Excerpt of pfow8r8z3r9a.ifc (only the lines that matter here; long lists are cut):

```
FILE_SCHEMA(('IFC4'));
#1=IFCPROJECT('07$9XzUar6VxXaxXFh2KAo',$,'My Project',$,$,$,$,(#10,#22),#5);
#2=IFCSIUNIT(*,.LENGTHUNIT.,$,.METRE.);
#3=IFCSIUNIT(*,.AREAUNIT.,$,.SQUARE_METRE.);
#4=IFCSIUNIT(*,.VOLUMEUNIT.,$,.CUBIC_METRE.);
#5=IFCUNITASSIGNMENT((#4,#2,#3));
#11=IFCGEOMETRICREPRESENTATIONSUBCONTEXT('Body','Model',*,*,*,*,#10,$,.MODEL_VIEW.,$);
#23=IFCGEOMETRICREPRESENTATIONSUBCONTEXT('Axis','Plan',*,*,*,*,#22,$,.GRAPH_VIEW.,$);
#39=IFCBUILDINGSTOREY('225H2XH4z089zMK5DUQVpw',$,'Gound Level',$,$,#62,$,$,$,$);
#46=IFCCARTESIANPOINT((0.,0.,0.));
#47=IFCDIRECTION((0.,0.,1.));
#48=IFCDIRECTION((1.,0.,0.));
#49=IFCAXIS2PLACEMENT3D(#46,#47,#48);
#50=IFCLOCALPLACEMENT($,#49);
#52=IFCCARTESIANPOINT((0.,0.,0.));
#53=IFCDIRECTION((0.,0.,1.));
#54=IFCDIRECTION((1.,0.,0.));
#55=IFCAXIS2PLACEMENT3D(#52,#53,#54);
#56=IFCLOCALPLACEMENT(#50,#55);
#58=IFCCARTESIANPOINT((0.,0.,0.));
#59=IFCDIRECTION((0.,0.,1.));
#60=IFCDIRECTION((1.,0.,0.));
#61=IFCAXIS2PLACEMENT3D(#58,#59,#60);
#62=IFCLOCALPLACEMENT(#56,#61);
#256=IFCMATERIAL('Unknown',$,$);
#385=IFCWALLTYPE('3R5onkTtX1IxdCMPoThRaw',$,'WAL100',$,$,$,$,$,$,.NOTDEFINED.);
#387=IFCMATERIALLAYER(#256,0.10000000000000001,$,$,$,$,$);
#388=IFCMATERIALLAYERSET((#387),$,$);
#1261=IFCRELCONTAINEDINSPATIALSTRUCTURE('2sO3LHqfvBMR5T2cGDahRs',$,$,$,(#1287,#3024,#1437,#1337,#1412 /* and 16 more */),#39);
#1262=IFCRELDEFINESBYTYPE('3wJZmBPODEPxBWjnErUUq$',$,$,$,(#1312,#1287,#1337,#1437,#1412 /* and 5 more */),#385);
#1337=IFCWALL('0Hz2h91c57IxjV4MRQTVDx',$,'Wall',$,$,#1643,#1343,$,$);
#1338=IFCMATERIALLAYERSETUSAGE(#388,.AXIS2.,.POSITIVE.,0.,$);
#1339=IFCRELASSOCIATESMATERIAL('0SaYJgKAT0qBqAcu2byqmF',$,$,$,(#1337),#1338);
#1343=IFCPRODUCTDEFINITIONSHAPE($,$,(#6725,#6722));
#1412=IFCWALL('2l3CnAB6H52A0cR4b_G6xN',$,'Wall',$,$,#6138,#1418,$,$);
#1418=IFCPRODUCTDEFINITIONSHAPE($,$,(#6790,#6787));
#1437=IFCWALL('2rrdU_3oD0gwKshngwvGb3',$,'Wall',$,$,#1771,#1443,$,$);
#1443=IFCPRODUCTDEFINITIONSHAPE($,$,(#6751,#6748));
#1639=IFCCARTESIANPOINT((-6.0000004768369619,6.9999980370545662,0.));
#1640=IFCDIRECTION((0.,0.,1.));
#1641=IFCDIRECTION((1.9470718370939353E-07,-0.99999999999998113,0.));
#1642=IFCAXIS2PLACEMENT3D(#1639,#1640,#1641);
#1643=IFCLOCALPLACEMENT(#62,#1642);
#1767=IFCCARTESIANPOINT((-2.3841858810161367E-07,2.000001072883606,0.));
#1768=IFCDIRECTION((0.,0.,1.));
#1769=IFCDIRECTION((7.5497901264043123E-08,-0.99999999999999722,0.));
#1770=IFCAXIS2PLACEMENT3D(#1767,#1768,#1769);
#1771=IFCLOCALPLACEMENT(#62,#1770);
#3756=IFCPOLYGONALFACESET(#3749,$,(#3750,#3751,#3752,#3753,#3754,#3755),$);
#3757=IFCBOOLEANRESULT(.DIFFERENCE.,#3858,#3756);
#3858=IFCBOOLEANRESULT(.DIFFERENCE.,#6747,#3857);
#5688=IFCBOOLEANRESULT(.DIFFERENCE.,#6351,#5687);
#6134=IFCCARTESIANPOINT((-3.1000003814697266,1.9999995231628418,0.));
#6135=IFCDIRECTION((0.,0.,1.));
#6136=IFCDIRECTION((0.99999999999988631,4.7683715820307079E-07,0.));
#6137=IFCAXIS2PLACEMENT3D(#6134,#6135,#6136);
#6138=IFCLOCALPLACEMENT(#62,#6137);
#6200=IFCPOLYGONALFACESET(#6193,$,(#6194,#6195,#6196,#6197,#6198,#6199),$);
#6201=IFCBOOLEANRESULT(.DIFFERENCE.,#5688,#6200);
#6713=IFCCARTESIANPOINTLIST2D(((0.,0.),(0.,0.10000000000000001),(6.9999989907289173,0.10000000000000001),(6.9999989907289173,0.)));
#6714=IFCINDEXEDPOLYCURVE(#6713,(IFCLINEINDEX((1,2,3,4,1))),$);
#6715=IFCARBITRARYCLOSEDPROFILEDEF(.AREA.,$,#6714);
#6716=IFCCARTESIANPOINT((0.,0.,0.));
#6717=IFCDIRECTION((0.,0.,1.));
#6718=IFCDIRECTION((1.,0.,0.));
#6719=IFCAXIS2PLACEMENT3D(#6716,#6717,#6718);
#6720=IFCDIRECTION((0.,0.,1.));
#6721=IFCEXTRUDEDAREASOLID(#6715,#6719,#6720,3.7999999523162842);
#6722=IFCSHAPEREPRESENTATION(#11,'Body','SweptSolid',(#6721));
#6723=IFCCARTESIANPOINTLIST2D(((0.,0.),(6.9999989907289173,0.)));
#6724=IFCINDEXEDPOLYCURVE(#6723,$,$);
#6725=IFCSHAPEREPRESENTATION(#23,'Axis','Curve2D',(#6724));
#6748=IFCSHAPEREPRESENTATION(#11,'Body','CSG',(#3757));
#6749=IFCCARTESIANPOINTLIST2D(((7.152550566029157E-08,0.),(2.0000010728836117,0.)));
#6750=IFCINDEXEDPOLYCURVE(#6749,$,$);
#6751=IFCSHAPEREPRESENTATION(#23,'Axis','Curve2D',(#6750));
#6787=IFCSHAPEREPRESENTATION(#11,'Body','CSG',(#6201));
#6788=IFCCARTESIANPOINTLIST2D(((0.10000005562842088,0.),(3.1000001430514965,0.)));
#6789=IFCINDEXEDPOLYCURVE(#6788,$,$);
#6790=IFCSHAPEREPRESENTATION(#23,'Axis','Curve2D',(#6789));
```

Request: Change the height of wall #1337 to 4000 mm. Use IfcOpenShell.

```python
import ifcopenshell
import ifcopenshell.geom
import ifcopenshell.util.representation
import ifcopenshell.util.shape

model = ifcopenshell.open("pfow8r8z3r9a.ifc")
settings = ifcopenshell.geom.settings()


def volume(element):
    """Net volume in cubic metres, openings subtracted."""
    shape = ifcopenshell.geom.create_shape(settings, element)
    return ifcopenshell.util.shape.get_volume(shape.geometry)


wall = model.by_guid("0Hz2h91c57IxjV4MRQTVDx")
before = volume(wall)

body = ifcopenshell.util.representation.get_representation(wall, "Model", "Body")
solid = body.Items[0]
old_height = solid.Depth
solid.Depth = 4.0
after = volume(wall)

print(f"height {old_height:g} -> {solid.Depth:g}, volume {before:.3f} -> {after:.3f} m3")

model.write("pfow8r8z3r9a_updated.ifc")
```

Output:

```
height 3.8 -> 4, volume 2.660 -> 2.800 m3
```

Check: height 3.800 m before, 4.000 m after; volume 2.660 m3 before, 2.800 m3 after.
